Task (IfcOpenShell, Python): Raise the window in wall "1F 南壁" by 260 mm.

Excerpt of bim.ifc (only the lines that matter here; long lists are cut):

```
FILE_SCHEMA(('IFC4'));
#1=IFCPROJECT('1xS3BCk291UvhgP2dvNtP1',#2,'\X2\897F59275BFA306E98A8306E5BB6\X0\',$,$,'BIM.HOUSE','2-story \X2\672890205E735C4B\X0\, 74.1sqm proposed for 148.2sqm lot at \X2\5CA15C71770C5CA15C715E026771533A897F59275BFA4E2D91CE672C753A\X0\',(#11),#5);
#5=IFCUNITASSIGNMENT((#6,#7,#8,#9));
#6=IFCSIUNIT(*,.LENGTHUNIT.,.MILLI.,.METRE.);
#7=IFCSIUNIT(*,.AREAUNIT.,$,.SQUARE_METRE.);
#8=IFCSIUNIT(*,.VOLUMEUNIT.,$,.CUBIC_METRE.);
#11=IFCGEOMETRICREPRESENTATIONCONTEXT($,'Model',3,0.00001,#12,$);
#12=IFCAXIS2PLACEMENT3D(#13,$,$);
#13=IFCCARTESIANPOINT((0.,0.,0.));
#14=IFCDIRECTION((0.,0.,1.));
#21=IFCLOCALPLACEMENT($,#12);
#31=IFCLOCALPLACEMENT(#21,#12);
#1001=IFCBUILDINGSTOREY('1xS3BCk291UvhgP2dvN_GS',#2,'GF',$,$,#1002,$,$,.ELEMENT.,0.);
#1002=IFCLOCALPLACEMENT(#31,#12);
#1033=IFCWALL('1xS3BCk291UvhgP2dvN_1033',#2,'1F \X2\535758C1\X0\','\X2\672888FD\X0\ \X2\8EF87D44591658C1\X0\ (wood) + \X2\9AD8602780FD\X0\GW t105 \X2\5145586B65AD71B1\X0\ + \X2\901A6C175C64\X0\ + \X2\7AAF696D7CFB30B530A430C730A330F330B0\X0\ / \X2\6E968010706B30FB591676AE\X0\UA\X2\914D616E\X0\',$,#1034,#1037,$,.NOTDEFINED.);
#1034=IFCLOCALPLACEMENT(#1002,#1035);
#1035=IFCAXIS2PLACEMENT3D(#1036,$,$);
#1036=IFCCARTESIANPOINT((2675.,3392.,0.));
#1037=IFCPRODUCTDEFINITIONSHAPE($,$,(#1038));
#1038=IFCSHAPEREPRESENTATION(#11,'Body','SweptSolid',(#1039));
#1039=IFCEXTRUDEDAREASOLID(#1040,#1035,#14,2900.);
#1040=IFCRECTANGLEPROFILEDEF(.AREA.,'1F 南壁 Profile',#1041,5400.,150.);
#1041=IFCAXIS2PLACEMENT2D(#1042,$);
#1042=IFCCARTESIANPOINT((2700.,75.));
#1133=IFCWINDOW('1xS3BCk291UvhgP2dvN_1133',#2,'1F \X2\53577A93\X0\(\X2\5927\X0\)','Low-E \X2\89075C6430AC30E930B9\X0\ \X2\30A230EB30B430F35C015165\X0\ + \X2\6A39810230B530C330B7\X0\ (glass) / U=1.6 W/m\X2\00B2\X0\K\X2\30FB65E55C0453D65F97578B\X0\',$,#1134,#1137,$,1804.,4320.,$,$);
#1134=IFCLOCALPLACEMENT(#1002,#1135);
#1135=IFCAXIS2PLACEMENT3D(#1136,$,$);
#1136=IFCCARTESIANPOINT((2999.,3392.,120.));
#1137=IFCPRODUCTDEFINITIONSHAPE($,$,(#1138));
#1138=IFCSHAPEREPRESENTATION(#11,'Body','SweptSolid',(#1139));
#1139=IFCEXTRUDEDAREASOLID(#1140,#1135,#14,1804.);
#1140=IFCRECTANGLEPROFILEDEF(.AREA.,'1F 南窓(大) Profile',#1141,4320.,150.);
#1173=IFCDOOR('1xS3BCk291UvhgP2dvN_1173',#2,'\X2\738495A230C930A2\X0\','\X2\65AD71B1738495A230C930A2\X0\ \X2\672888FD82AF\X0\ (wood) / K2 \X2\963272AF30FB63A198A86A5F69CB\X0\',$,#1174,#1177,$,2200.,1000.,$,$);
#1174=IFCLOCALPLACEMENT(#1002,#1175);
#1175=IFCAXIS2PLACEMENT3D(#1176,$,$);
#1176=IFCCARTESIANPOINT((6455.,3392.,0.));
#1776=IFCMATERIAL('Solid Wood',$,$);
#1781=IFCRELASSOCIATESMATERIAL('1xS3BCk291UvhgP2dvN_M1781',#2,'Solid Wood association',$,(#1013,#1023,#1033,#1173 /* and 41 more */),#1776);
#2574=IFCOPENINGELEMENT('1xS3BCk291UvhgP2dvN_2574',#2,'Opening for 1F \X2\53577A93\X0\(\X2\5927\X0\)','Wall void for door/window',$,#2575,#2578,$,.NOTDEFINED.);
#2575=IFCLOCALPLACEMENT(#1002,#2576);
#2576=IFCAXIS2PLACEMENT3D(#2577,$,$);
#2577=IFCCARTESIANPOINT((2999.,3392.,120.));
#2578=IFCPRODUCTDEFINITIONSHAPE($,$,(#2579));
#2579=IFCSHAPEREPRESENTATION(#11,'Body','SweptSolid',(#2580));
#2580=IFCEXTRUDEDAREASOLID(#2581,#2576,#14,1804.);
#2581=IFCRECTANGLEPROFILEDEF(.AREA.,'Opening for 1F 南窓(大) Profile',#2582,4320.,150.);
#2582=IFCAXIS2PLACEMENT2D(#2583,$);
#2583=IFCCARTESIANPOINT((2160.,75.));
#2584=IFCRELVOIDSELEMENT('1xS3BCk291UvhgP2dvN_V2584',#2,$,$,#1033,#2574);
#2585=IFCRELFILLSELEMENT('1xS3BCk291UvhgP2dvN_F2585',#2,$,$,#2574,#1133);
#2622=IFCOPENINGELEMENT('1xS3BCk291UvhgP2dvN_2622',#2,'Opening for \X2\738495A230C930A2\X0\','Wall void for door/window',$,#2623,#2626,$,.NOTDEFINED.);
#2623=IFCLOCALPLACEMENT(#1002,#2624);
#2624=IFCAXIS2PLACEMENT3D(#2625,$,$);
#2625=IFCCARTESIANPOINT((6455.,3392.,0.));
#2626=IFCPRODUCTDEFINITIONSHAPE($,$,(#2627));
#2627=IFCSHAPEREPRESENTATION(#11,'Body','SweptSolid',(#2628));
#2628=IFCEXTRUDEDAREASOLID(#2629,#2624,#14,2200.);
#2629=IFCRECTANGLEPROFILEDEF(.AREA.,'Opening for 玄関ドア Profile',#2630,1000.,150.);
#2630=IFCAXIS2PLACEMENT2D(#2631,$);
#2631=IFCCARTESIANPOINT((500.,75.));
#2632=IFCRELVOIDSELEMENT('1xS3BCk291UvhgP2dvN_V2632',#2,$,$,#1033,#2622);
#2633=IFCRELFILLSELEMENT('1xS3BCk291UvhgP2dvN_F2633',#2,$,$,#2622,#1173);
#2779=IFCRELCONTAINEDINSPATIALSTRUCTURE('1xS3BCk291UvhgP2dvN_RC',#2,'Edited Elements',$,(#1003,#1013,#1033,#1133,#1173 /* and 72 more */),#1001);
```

```python
import numpy as np
import ifcopenshell
import ifcopenshell.api.geometry
import ifcopenshell.util.placement
import ifcopenshell.util.unit

model = ifcopenshell.open("bim.ifc")
unit_scale = ifcopenshell.util.unit.calculate_unit_scale(model)

window = model.by_guid("1xS3BCk291UvhgP2dvN_1133")
opening = window.FillsVoids[0].RelatingOpeningElement
dz = 260.0

shift = np.array([0.0, 0.0, dz])
# The window is not placed relative to its opening, so move both.
for product in (opening, window):
    matrix = ifcopenshell.util.placement.get_local_placement(product.ObjectPlacement)
    matrix[:3, 3] += shift
    ifcopenshell.api.geometry.edit_object_placement(model, product=product, matrix=matrix, is_si=False)

print(f"moved by {dz * unit_scale:+.3f} m")

model.write("bim-out.ifc")
```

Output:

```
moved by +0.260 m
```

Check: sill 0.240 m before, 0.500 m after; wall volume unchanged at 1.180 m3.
